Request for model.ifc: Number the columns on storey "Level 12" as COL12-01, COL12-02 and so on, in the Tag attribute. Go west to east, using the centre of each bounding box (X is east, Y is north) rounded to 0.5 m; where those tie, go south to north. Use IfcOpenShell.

First a look at what the model holds.

```python
import ifcopenshell
import ifcopenshell.util.element
import ifcopenshell.util.placement

model = ifcopenshell.open("model.ifc")
print(model.schema)
storey = next(s for s in model.by_type("IfcBuildingStorey") if s.Name == "Level 12")
columns = [e for e in ifcopenshell.util.element.get_decomposition(storey) if e.is_a("IfcColumn")]
for e in sorted(columns, key=lambda e: e.id()):
    origin = ifcopenshell.util.placement.get_local_placement(e.ObjectPlacement)[:3, 3]
    print(e.id(), e.Tag, e.Name, origin.round(2) + 0.0, sep=" | ")
```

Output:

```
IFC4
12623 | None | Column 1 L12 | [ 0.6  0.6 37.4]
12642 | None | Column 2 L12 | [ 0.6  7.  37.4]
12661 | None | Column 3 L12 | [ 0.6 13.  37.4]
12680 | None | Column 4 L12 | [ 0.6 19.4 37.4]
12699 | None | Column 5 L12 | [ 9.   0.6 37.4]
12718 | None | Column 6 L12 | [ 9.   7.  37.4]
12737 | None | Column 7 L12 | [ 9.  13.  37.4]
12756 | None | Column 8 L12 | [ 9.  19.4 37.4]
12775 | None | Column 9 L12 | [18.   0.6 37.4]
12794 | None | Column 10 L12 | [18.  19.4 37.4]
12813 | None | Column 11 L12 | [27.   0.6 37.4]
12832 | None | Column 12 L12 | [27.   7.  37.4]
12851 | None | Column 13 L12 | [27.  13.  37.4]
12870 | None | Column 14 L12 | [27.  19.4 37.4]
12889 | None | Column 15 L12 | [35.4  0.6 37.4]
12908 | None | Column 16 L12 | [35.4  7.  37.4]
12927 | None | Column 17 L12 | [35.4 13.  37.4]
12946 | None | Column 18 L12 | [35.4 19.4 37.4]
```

```python
import ifcopenshell
import ifcopenshell.geom
import ifcopenshell.util.element
import ifcopenshell.util.shape

model = ifcopenshell.open("model.ifc")
settings = ifcopenshell.geom.settings()
settings.set("use-world-coords", True)


def centre(element):
    shape = ifcopenshell.geom.create_shape(settings, element)
    return ifcopenshell.util.shape.get_bbox_centroid(shape.geometry)


storey = next(s for s in model.by_type("IfcBuildingStorey") if s.Name == "Level 12")
columns = [e for e in ifcopenshell.util.element.get_decomposition(storey) if e.is_a("IfcColumn")]

# Insertion points can sit at a corner or the storey origin, so sort by the geometry (in metres).
centres = {e: centre(e) for e in columns}
columns.sort(key=lambda e: (round(centres[e][0] / 0.5), centres[e][1]))

for i, e in enumerate(columns, start=1):
    number = f"COL12-{i:02d}"
    e.Tag = number
    print(e.id(), number)

model.write("model-out.ifc")
```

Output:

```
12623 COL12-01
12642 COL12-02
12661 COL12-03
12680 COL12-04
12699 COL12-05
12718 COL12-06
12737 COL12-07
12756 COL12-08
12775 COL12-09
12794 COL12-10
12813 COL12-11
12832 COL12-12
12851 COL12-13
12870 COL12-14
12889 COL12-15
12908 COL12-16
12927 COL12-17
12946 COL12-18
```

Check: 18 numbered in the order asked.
